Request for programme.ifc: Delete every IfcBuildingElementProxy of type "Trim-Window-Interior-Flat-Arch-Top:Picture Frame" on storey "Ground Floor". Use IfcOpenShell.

First a look at what the model holds.

```python
import ifcopenshell
import ifcopenshell.util.element

model = ifcopenshell.open("programme.ifc")
print(model.schema)
storey = next(s for s in model.by_type("IfcBuildingStorey") if s.Name == "Ground Floor")
proxies = [e for e in ifcopenshell.util.element.get_decomposition(storey) if e.is_a("IfcBuildingElementProxy")]
seen = {}
for e in proxies:
    element_type = ifcopenshell.util.element.get_type(e)
    name = element_type.Name if element_type not in (None, e) else None
    seen[name] = seen.get(name, 0) + 1
for name, count in sorted(seen.items(), key=str):
    print(count, "x", name)
```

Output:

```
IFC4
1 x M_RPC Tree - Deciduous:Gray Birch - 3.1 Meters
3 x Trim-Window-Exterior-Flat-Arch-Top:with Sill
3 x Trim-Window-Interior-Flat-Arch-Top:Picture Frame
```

```python
import ifcopenshell
import ifcopenshell.api.root
import ifcopenshell.util.element

model = ifcopenshell.open("programme.ifc")

storey = next(s for s in model.by_type("IfcBuildingStorey") if s.Name == "Ground Floor")
proxies = [e for e in ifcopenshell.util.element.get_decomposition(storey) if e.is_a("IfcBuildingElementProxy")]
targets = [e for e in proxies if (t := ifcopenshell.util.element.get_type(e)) not in (None, e) and t.Name == "Trim-Window-Interior-Flat-Arch-Top:Picture Frame"]

for e in targets:
    ifcopenshell.api.root.remove_product(model, product=e)
print(len(targets), "removed")

model.write("programme_v2.ifc")
```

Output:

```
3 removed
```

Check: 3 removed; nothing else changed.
